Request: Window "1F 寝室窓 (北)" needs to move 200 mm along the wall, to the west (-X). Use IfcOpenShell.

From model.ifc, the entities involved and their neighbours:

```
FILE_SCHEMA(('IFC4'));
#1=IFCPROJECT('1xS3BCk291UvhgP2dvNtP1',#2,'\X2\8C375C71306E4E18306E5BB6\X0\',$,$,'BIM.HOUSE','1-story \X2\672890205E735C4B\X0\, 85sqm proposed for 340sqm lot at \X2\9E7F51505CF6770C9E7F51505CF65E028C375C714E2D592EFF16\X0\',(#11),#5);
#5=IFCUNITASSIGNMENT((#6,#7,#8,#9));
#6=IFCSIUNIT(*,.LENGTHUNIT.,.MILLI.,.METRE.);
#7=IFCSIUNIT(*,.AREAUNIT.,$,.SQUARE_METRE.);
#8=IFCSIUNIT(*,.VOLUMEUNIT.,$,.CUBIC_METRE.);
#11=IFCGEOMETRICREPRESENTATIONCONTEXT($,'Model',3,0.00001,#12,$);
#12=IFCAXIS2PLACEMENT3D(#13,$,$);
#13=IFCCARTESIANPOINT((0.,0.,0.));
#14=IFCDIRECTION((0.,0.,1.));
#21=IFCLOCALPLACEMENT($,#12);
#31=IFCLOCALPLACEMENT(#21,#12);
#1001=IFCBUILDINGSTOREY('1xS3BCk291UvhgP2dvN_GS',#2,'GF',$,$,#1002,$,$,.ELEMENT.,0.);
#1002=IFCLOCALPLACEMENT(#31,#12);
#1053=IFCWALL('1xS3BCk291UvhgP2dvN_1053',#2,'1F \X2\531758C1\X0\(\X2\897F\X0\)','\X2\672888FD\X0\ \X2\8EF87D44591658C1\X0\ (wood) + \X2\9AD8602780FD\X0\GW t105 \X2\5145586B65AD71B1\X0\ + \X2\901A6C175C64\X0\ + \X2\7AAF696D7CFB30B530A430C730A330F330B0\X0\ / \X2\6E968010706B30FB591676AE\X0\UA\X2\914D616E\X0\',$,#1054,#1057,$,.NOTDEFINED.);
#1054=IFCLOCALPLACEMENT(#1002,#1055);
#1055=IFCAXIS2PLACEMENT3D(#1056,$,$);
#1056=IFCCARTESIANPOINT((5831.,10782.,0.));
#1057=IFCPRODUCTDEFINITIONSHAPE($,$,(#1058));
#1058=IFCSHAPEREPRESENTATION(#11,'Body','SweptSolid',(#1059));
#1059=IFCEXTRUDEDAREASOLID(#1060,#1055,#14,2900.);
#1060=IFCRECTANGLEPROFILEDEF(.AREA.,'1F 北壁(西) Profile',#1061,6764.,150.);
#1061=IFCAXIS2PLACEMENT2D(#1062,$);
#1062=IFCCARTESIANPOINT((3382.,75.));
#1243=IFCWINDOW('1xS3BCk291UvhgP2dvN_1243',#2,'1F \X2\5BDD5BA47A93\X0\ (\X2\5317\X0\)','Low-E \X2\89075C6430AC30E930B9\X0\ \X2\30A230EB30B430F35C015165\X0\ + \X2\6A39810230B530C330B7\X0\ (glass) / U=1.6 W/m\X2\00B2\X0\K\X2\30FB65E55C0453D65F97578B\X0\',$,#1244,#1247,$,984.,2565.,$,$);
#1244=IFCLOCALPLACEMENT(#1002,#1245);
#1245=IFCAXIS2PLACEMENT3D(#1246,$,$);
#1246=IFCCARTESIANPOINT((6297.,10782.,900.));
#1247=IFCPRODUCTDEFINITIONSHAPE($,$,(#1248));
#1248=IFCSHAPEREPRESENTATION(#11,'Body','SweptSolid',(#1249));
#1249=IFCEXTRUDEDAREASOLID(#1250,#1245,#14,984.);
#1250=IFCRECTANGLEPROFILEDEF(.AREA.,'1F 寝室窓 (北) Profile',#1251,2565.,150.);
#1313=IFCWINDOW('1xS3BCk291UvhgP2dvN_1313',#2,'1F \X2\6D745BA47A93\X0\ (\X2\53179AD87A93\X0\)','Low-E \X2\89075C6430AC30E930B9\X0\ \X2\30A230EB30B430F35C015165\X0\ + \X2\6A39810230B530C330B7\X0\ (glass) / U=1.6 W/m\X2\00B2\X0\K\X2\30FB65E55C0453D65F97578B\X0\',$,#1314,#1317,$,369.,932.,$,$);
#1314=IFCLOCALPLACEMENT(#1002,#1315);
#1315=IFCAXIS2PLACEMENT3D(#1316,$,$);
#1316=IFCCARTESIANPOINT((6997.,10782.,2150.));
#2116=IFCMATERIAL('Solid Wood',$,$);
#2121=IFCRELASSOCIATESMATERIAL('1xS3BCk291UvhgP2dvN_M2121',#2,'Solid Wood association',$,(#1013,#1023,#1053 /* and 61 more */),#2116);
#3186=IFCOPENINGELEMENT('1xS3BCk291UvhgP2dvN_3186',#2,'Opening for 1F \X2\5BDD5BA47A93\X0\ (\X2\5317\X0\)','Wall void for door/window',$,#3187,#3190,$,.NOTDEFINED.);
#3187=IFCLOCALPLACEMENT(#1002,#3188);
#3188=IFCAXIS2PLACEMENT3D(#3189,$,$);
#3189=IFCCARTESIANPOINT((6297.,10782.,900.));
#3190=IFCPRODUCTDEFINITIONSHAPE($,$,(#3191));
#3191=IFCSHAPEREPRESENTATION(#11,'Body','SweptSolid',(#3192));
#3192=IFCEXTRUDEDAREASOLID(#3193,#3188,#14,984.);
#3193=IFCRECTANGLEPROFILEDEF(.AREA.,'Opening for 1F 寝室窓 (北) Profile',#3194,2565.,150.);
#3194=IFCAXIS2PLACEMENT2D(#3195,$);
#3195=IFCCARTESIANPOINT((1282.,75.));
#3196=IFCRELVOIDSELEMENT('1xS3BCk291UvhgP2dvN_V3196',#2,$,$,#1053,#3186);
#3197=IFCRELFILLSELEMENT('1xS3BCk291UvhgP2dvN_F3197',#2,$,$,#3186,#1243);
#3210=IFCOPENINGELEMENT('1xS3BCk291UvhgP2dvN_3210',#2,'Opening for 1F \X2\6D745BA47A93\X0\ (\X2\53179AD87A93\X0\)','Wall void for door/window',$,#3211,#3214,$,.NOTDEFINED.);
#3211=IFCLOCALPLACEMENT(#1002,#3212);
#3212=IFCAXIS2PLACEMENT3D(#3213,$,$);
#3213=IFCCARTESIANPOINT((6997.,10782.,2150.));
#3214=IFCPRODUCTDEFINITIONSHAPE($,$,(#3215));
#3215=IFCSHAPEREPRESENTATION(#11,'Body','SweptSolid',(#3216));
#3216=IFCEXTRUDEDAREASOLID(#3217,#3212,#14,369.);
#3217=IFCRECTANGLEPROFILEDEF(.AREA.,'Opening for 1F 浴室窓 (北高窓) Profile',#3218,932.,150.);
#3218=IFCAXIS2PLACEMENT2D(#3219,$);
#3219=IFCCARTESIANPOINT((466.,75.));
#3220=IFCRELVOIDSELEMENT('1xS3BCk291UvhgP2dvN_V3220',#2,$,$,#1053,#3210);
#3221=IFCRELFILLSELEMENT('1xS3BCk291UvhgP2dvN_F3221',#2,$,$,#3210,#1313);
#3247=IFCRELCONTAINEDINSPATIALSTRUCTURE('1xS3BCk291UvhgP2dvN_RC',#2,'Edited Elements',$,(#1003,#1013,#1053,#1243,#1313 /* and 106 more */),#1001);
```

```python
import ifcopenshell
import ifcopenshell.api.geometry
import ifcopenshell.util.placement

model = ifcopenshell.open("model.ifc")

window = model.by_guid("1xS3BCk291UvhgP2dvN_1243")
opening = window.FillsVoids[0].RelatingOpeningElement
wall = opening.VoidsElements[0].RelatingBuildingElement

wall_matrix = ifcopenshell.util.placement.get_local_placement(wall.ObjectPlacement)
shift = wall_matrix[:3, 0] * -200.0
before = ifcopenshell.util.placement.get_local_placement(window.ObjectPlacement)[:3, 3].copy()

# The window is not placed relative to its opening, so move both.
for product in (opening, window):
    matrix = ifcopenshell.util.placement.get_local_placement(product.ObjectPlacement)
    matrix[:3, 3] += shift
    ifcopenshell.api.geometry.edit_object_placement(model, product=product, matrix=matrix, is_si=False)

after = ifcopenshell.util.placement.get_local_placement(window.ObjectPlacement)[:3, 3]
print("window moved by", (after - before).round(3) + 0.0)

model.write("model-out.ifc")
```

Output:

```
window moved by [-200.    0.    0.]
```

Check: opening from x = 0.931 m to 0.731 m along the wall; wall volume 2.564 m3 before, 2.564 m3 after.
